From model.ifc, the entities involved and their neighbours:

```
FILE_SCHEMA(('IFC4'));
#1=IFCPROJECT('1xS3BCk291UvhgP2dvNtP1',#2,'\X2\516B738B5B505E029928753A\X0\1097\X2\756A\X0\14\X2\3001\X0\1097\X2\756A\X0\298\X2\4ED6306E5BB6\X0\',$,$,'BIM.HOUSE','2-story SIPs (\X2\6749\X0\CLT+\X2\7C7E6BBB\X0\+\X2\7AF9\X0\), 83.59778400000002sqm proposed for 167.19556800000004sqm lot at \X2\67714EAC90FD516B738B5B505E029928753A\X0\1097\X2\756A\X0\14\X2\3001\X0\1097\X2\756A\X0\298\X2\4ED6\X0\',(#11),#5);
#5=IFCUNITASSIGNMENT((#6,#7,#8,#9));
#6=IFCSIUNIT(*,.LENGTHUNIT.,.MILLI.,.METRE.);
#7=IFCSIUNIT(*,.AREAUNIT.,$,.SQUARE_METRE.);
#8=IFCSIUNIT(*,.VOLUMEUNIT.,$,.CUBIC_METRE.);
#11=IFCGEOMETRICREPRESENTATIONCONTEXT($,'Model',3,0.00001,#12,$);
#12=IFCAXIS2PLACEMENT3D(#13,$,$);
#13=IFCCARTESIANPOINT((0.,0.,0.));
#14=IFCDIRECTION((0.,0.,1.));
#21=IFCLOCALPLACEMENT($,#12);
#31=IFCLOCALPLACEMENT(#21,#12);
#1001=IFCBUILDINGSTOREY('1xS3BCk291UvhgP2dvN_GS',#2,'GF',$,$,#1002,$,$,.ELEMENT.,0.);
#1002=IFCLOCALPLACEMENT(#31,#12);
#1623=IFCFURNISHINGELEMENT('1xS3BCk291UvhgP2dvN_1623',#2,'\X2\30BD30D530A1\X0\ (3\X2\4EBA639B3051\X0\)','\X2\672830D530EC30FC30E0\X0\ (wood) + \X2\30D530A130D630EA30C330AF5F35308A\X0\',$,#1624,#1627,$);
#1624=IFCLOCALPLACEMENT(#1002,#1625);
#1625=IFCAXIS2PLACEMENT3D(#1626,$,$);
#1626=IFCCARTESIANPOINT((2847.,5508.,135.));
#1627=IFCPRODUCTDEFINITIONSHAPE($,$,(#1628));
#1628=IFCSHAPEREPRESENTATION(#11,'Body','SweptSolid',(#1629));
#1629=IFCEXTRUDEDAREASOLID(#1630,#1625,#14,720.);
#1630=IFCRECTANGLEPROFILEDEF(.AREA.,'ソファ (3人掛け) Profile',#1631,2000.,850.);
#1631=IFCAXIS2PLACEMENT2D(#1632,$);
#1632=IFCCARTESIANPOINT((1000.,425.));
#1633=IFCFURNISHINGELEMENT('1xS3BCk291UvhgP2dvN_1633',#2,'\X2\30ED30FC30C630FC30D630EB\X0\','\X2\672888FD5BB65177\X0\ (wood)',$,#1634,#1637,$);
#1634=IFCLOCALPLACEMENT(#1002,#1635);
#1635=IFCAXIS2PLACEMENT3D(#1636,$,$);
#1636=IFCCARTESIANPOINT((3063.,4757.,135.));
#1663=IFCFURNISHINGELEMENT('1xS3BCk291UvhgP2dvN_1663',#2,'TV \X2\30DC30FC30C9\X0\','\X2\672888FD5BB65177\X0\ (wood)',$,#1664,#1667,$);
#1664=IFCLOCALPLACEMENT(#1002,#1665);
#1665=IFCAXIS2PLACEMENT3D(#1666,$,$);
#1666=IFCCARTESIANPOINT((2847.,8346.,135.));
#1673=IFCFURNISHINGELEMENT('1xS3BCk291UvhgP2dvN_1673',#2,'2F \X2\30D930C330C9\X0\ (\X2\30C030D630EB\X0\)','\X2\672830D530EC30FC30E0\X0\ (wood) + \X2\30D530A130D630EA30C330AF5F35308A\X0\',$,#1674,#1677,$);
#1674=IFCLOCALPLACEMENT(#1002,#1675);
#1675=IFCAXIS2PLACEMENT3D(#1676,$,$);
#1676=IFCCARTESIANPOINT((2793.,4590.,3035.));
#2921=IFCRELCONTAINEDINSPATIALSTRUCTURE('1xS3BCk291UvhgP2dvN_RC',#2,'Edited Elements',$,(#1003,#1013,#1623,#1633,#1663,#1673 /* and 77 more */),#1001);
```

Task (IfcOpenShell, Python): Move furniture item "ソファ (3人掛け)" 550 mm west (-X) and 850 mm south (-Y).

```python
import ifcopenshell
import ifcopenshell.api.geometry
import ifcopenshell.util.placement
import ifcopenshell.util.unit

model = ifcopenshell.open("model.ifc")
unit_scale = ifcopenshell.util.unit.calculate_unit_scale(model)

item = model.by_guid("1xS3BCk291UvhgP2dvN_1623")
matrix = ifcopenshell.util.placement.get_local_placement(item.ObjectPlacement)
matrix[0, 3] -= 0.55 / unit_scale
matrix[1, 3] -= 0.85 / unit_scale
ifcopenshell.api.geometry.edit_object_placement(model, product=item, matrix=matrix, is_si=False)

print(ifcopenshell.util.placement.get_local_placement(item.ObjectPlacement).round(3) + 0.0)

model.write("model_v2.ifc")
```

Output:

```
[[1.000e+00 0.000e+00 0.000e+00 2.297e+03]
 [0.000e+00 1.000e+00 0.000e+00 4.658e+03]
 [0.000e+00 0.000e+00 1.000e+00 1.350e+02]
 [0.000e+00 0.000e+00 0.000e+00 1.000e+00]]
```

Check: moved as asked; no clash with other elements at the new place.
